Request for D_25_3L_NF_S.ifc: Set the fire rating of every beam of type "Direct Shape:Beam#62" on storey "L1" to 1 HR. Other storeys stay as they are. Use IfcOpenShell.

First a look at what the model holds.

```python
import ifcopenshell
import ifcopenshell.util.element

model = ifcopenshell.open("D_25_3L_NF_S.ifc")
print(model.schema)
storey = next(s for s in model.by_type("IfcBuildingStorey") if s.Name == "L1")
beams = [e for e in ifcopenshell.util.element.get_decomposition(storey) if e.is_a("IfcBeam")]
seen = {}
for e in beams:
    element_type = ifcopenshell.util.element.get_type(e)
    key = (element_type.Name if element_type != e and element_type else None, ifcopenshell.util.element.get_pset(e, "Pset_BeamCommon", "FireRating"))
    seen[key] = seen.get(key, 0) + 1
for (name, value), count in sorted(seen.items(), key=str):
    print(count, "x", name, "|", value)
```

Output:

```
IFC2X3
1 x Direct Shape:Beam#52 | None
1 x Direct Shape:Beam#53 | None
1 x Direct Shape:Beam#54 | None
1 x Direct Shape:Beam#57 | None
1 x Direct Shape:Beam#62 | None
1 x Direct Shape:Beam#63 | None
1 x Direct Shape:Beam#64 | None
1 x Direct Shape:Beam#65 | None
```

```python
import ifcopenshell
import ifcopenshell.api.pset
import ifcopenshell.util.element

model = ifcopenshell.open("D_25_3L_NF_S.ifc")

storey = next(s for s in model.by_type("IfcBuildingStorey") if s.Name == "L1")
beams = [e for e in ifcopenshell.util.element.get_decomposition(storey) if e.is_a("IfcBeam")]

count = 0
for e in beams:
    element_type = ifcopenshell.util.element.get_type(e)
    if element_type in (None, e) or element_type.Name != "Direct Shape:Beam#62":
        continue
    # add_pset returns the element's existing set when there is one.
    pset = ifcopenshell.api.pset.add_pset(model, product=e, name="Pset_BeamCommon")
    ifcopenshell.api.pset.edit_pset(model, pset=pset, properties={"FireRating": "1 HR"})
    count += 1

print(count, "beams updated")

model.write("D_25_3L_NF_S_edited.ifc")
```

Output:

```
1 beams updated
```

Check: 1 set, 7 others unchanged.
